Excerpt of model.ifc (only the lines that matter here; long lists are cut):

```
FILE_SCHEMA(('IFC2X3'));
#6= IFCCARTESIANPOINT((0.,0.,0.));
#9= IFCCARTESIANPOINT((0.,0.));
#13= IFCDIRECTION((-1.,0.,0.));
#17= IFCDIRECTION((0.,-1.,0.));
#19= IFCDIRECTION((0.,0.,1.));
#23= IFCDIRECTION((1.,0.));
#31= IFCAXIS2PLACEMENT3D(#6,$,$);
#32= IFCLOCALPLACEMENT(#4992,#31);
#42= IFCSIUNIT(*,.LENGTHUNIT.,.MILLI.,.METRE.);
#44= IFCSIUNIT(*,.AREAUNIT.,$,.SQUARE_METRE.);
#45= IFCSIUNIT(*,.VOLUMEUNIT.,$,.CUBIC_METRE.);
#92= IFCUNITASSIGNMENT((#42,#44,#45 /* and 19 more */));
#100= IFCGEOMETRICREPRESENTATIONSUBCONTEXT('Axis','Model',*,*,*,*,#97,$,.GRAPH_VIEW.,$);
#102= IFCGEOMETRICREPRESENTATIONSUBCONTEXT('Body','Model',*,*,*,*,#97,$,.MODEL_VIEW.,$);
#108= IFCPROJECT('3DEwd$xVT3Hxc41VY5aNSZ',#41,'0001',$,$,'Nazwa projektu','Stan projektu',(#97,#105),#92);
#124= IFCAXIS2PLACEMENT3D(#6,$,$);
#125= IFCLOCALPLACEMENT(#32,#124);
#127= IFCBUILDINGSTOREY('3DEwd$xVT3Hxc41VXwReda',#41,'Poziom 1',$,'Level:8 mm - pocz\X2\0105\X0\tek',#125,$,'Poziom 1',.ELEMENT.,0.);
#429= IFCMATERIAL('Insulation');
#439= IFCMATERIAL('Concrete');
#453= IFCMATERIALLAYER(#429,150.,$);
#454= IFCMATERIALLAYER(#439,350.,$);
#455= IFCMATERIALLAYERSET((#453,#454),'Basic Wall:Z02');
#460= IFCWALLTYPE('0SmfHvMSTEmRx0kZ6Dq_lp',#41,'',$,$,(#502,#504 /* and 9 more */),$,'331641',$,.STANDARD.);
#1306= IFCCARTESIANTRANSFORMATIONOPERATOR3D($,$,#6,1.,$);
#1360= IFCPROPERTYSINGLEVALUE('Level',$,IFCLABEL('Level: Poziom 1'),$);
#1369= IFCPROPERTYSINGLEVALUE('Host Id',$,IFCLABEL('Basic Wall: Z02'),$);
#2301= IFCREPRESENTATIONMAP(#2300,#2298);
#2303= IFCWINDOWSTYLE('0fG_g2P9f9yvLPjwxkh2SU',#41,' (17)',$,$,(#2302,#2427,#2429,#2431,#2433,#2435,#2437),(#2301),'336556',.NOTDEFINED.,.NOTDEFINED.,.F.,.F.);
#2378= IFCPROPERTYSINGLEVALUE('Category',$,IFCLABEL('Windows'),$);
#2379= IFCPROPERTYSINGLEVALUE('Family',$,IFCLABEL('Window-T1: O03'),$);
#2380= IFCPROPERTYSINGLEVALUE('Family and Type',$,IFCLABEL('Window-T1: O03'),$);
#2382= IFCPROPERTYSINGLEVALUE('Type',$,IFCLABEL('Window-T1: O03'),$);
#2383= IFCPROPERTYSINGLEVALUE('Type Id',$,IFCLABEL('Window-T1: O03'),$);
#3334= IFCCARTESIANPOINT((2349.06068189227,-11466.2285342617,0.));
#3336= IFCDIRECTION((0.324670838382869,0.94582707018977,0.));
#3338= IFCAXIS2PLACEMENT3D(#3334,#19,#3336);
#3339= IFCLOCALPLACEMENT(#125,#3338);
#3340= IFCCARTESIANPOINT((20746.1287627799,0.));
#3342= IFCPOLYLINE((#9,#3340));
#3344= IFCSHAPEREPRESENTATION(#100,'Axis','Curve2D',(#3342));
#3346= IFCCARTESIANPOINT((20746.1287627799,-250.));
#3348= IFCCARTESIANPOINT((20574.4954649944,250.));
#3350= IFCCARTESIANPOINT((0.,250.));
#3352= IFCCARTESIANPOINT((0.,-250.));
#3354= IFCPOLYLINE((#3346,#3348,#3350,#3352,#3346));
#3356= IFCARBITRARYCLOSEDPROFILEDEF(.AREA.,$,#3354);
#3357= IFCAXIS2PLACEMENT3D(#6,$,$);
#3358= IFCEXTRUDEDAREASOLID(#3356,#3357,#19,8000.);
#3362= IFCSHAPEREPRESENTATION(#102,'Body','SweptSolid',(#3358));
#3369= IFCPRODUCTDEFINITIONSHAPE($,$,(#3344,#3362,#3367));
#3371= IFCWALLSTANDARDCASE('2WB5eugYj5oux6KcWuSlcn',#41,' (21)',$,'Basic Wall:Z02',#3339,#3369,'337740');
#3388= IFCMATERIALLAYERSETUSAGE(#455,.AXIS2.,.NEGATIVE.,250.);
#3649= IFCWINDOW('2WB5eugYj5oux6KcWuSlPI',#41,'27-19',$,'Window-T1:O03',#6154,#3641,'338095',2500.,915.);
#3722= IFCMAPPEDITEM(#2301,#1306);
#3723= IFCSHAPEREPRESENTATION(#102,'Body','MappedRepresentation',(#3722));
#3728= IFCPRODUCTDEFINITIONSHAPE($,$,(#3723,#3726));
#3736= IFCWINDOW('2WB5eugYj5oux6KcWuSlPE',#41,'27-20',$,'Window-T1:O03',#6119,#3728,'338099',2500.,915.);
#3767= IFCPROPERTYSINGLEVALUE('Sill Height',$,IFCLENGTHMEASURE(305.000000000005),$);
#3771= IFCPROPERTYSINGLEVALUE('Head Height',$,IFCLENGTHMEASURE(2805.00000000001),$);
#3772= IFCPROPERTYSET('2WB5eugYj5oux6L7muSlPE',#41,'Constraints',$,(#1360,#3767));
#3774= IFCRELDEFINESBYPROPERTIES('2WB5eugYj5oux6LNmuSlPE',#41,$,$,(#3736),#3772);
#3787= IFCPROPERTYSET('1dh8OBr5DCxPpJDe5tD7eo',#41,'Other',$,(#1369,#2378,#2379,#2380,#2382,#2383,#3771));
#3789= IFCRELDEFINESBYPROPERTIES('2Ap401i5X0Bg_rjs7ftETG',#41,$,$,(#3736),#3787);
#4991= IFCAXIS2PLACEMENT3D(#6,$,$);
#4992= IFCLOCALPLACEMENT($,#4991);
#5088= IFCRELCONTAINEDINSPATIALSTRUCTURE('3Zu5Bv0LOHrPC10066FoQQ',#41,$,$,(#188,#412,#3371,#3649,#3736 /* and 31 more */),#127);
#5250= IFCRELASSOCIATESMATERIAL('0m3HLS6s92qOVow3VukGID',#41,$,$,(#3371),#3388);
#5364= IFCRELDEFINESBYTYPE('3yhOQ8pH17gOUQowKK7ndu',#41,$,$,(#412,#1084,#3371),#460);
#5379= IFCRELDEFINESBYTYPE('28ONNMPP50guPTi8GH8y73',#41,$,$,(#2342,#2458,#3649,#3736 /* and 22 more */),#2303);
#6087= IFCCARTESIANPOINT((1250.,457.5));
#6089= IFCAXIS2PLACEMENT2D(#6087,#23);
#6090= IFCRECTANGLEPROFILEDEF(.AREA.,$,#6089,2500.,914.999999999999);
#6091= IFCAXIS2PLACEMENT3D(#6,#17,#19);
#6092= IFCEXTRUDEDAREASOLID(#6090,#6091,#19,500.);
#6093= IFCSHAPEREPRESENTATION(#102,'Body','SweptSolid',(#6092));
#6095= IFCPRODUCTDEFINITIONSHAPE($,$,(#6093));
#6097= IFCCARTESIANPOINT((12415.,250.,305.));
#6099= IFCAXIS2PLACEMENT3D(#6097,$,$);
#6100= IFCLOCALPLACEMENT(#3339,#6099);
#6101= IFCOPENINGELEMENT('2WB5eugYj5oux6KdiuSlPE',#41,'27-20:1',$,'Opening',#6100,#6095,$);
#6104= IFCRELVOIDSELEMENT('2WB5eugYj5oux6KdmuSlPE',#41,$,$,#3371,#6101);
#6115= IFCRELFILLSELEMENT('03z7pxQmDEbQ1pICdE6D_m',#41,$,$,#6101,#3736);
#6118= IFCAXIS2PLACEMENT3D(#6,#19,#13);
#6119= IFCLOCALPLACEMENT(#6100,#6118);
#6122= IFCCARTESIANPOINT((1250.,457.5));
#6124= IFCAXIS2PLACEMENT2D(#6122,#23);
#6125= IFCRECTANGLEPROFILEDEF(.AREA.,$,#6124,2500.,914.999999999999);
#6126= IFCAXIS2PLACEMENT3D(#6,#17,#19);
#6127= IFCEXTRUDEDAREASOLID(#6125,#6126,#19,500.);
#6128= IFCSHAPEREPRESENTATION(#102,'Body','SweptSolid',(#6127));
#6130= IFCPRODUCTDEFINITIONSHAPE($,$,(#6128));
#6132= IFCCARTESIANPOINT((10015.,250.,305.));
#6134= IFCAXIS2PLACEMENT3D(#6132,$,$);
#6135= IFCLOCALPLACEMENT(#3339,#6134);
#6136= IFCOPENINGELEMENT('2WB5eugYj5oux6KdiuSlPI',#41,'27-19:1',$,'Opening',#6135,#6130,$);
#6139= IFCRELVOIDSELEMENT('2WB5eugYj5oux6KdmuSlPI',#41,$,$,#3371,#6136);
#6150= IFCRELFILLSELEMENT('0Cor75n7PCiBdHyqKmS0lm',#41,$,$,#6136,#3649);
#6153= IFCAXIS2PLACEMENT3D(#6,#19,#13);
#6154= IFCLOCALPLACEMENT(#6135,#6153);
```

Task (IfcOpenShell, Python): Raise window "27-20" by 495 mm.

```python
import numpy as np
import ifcopenshell
import ifcopenshell.api.geometry
import ifcopenshell.api.pset
import ifcopenshell.util.element
import ifcopenshell.util.placement
import ifcopenshell.util.unit

model = ifcopenshell.open("model.ifc")
unit_scale = ifcopenshell.util.unit.calculate_unit_scale(model)

window = model.by_guid("2WB5eugYj5oux6KcWuSlPE")
opening = window.FillsVoids[0].RelatingOpeningElement
dz = 495.0

shift = np.array([0.0, 0.0, dz])
# The window is placed relative to its opening, so it follows when the opening moves.
matrix = ifcopenshell.util.placement.get_local_placement(opening.ObjectPlacement)
matrix[:3, 3] += shift
ifcopenshell.api.geometry.edit_object_placement(
    model, product=opening, matrix=matrix, is_si=False, should_transform_children=True
)

# Keep the stored heights in step.
pset = model.by_id(ifcopenshell.util.element.get_pset(window, "Constraints", should_inherit=False)["id"])
ifcopenshell.api.pset.edit_pset(model, pset=pset, properties={
    "Sill Height": model.create_entity("IfcLengthMeasure", ifcopenshell.util.element.get_pset(window, "Constraints", "Sill Height") + dz),
})
pset = model.by_id(ifcopenshell.util.element.get_pset(window, "Other", should_inherit=False)["id"])
ifcopenshell.api.pset.edit_pset(model, pset=pset, properties={
    "Head Height": model.create_entity("IfcLengthMeasure", ifcopenshell.util.element.get_pset(window, "Other", "Head Height") + dz),
})

print(f"moved by {dz * unit_scale:+.3f} m")

model.write("model_rev.ifc")
```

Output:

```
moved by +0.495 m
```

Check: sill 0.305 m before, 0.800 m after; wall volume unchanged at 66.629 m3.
